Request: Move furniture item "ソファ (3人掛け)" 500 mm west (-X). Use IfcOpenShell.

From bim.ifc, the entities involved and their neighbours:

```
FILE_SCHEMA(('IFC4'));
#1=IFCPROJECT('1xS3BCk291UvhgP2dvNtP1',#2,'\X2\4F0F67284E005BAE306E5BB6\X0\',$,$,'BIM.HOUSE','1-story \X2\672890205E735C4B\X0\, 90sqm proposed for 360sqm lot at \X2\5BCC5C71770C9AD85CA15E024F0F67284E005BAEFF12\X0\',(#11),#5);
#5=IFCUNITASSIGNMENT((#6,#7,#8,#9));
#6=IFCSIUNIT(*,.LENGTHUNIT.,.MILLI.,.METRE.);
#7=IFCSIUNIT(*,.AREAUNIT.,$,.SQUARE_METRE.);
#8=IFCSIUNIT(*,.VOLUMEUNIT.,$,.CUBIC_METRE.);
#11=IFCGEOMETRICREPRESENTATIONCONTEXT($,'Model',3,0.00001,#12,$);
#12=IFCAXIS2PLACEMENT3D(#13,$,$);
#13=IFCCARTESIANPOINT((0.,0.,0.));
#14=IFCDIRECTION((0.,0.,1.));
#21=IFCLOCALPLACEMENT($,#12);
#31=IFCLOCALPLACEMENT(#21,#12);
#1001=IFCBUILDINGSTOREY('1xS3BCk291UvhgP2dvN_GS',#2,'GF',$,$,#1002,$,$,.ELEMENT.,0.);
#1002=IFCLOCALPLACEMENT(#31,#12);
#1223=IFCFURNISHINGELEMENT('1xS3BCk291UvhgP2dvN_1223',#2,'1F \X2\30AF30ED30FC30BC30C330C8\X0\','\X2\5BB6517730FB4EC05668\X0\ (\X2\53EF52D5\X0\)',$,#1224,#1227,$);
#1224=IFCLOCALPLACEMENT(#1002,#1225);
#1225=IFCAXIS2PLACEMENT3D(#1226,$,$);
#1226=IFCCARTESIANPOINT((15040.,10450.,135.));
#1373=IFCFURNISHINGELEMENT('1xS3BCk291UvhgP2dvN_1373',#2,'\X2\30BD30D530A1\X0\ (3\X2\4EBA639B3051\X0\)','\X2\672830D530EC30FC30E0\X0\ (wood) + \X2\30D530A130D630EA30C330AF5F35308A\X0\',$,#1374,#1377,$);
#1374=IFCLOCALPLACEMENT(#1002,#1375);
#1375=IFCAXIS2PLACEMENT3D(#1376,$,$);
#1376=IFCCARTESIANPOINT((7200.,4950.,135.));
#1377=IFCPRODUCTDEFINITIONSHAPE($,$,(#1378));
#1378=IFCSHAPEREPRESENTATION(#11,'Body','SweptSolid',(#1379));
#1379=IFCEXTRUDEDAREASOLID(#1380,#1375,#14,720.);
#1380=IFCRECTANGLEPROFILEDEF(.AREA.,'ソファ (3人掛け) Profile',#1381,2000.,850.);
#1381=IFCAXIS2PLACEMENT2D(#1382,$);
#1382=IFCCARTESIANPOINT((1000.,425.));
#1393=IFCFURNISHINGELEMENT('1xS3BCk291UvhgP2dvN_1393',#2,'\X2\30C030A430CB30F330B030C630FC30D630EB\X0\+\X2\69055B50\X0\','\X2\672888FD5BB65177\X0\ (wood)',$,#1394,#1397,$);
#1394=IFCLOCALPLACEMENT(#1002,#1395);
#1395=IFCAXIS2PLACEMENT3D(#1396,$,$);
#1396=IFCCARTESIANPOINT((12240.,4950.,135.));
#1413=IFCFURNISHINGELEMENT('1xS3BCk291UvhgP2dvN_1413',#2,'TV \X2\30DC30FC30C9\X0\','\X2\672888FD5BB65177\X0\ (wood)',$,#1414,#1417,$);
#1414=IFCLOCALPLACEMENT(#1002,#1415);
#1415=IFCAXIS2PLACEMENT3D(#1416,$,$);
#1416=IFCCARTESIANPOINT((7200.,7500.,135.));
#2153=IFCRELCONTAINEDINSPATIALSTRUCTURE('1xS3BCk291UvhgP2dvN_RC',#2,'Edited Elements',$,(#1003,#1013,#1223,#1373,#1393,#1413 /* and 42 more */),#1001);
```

```python
import ifcopenshell
import ifcopenshell.api.geometry
import ifcopenshell.util.placement
import ifcopenshell.util.unit

model = ifcopenshell.open("bim.ifc")
unit_scale = ifcopenshell.util.unit.calculate_unit_scale(model)

item = model.by_id(1373)
matrix = ifcopenshell.util.placement.get_local_placement(item.ObjectPlacement)
matrix[0, 3] -= 0.5 / unit_scale
ifcopenshell.api.geometry.edit_object_placement(model, product=item, matrix=matrix, is_si=False)

print(ifcopenshell.util.placement.get_local_placement(item.ObjectPlacement).round(3) + 0.0)

model.write("bim_edited.ifc")
```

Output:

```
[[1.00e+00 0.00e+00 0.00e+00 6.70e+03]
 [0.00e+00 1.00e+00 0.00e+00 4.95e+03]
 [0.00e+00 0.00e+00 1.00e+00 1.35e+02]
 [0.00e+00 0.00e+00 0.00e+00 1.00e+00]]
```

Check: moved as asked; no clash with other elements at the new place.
